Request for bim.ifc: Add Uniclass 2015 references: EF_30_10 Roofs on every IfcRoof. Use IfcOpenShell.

First a look at what the model holds.

```python
import ifcopenshell

model = ifcopenshell.open("bim.ifc")
print(model.schema)
print("classifications:", [c.Name for c in model.by_type("IfcClassification")])
for ifc_class in ("IfcDoor", "IfcRoof", "IfcStair", "IfcWall", "IfcWindow"):
    print(ifc_class, len(model.by_type(ifc_class)))
```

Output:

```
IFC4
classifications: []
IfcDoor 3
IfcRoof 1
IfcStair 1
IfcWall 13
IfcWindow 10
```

```python
import ifcopenshell
import ifcopenshell.api.classification

model = ifcopenshell.open("bim.ifc")

system = ifcopenshell.api.classification.add_classification(model, classification="Uniclass 2015")

codes = {
    "IfcRoof": ("EF_30_10", "Roofs"),
}
for ifc_class, (code, name) in codes.items():
    products = model.by_type(ifc_class)
    ifcopenshell.api.classification.add_reference(
        model, products=products, classification=system, identification=code, name=name
    )
    print(code, len(products))

model.write("bim_rev.ifc")
```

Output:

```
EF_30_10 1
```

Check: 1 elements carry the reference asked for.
